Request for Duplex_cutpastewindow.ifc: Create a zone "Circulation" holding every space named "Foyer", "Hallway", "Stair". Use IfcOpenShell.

First a look at what the model holds.

```python
import ifcopenshell

model = ifcopenshell.open("Duplex_cutpastewindow.ifc")
print(model.schema)
seen = {}
for space in model.by_type("IfcSpace"):
    seen[space.LongName] = seen.get(space.LongName, 0) + 1
for name, count in sorted(seen.items(), key=str):
    print(count, "x", name)
print("zones:", [z.Name for z in model.by_type("IfcZone")][:20])
```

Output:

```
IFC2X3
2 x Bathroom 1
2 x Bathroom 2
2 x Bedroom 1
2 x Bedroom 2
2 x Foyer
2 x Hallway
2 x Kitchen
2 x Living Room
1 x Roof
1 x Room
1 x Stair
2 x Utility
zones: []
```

```python
import ifcopenshell
import ifcopenshell.api.group
import ifcopenshell.api.root

model = ifcopenshell.open("Duplex_cutpastewindow.ifc")

names = {"Foyer", "Hallway", "Stair"}
spaces = [s for s in model.by_type("IfcSpace") if s.LongName in names]

zone = ifcopenshell.api.root.create_entity(model, ifc_class="IfcZone", name="Circulation")
ifcopenshell.api.group.assign_group(model, products=spaces, group=zone)
print(len(spaces), "spaces in", zone.Name)

model.write("Duplex_cutpastewindow_v2.ifc")
```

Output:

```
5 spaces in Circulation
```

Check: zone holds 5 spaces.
